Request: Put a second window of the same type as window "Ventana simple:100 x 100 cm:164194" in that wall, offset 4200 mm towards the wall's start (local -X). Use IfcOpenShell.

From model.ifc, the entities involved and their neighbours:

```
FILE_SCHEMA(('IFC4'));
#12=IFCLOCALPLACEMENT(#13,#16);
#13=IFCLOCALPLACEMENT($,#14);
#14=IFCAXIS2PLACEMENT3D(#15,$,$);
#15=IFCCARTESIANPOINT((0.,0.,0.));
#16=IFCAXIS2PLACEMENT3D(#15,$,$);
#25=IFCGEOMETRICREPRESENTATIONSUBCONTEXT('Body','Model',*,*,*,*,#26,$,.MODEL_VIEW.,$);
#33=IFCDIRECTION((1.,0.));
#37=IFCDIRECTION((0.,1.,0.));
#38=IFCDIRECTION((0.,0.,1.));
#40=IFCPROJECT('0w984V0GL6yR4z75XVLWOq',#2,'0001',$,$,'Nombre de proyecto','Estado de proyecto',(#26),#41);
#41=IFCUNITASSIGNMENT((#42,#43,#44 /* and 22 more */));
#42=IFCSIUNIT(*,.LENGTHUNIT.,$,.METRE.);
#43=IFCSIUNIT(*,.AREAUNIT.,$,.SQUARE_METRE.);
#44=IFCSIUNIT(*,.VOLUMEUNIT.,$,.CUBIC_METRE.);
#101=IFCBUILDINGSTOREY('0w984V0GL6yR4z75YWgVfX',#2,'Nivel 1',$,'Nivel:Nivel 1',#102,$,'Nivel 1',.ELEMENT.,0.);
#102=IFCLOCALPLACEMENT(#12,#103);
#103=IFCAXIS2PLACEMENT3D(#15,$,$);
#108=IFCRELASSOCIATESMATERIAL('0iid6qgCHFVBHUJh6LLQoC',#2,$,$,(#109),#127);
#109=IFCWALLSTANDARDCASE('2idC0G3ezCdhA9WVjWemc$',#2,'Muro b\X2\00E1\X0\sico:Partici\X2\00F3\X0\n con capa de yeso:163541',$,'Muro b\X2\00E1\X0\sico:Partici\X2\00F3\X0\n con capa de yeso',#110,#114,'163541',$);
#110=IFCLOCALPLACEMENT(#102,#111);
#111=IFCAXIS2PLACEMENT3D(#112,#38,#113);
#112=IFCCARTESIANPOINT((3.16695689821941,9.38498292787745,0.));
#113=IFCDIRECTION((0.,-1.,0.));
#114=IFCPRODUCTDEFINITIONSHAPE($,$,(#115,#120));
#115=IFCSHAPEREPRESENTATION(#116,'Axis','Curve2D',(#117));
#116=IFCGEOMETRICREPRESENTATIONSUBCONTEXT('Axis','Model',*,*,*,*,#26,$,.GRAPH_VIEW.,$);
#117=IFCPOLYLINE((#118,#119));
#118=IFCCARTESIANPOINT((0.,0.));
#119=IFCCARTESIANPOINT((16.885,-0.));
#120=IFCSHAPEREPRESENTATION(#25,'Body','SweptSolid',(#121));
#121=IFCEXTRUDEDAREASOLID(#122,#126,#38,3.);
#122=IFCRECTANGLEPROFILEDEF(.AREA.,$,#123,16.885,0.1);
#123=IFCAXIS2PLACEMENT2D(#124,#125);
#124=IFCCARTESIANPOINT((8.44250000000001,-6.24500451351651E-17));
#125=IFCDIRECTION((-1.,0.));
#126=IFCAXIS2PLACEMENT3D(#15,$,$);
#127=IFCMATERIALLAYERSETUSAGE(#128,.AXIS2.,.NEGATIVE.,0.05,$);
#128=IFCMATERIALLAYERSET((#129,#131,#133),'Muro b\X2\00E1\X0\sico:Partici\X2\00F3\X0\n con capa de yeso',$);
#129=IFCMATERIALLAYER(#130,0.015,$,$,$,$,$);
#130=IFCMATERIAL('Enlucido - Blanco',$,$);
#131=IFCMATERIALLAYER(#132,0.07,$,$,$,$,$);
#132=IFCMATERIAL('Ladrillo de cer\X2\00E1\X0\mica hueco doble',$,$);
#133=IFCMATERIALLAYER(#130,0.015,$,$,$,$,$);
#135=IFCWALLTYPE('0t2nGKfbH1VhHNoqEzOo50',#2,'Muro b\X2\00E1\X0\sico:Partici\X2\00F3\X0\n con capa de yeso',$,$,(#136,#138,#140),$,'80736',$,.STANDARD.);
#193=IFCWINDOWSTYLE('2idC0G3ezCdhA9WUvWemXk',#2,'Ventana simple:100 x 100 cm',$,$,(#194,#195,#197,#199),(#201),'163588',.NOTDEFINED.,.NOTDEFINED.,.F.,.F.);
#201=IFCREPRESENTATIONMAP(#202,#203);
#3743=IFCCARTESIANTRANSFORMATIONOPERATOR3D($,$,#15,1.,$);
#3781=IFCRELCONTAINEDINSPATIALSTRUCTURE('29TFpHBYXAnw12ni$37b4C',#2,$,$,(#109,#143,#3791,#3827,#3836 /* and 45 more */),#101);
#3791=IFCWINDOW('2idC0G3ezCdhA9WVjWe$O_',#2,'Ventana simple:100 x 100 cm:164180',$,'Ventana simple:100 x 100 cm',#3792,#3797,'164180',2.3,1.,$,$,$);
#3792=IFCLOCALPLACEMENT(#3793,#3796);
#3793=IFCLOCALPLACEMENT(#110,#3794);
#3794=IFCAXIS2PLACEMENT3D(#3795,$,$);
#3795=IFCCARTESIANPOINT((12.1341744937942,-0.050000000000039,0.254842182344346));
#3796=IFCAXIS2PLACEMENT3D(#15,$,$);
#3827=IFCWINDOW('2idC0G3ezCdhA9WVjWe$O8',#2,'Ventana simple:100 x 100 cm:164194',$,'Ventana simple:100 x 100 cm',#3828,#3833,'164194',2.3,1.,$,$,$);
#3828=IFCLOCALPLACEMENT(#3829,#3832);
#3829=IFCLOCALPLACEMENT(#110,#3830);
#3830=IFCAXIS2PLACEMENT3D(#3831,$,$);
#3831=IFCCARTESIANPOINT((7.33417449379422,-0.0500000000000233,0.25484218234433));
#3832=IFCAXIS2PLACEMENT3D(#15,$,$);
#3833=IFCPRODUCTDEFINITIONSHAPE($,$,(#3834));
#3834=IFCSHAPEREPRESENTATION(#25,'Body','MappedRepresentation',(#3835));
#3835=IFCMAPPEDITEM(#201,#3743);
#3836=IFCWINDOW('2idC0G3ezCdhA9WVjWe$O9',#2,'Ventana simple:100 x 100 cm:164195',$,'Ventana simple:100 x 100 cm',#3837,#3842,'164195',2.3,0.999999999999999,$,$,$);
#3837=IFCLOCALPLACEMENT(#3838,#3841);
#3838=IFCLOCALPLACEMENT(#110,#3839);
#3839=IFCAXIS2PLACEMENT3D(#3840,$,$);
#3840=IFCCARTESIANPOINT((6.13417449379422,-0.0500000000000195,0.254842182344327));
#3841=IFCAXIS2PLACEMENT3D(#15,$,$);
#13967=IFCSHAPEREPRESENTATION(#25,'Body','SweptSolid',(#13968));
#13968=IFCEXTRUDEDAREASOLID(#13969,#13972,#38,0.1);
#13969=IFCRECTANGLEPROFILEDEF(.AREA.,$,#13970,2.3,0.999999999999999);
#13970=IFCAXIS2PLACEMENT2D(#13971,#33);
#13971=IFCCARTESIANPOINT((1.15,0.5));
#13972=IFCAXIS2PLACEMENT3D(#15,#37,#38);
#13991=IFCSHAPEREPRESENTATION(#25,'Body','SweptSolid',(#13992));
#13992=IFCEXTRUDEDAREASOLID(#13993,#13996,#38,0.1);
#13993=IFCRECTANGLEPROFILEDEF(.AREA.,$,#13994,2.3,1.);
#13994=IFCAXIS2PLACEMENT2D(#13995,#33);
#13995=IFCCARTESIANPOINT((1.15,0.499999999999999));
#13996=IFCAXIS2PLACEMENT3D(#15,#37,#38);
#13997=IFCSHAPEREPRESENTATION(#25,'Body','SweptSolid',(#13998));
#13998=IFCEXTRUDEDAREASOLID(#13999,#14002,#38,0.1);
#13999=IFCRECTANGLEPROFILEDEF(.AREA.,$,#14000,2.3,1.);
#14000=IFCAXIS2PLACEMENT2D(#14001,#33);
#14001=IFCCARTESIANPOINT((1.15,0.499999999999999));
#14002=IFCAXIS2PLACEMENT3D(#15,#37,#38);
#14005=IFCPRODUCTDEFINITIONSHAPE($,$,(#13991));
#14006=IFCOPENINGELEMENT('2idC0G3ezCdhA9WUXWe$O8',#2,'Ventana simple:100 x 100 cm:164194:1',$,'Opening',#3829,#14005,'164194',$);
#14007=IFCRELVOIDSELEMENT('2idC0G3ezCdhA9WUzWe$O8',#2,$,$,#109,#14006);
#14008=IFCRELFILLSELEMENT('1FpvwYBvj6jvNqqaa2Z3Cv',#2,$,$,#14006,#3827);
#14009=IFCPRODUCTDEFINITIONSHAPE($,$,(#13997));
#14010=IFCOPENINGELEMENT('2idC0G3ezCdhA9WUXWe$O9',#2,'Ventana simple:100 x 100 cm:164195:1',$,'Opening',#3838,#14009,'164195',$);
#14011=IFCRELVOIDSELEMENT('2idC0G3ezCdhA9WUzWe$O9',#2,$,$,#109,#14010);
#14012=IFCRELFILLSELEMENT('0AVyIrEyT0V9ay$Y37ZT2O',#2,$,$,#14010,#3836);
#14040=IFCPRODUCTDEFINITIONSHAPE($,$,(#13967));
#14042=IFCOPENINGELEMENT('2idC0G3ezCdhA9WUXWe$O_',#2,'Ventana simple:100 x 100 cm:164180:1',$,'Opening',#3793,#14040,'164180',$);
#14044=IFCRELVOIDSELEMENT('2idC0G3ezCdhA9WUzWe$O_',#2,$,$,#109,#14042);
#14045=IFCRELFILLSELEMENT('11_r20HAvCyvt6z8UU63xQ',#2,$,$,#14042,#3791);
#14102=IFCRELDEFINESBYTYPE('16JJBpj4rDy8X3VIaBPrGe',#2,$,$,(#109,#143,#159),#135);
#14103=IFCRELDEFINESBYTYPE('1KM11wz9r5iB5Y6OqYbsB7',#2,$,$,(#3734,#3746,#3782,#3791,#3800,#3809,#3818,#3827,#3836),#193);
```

```python
import ifcopenshell
import ifcopenshell.api.feature
import ifcopenshell.api.geometry
import ifcopenshell.api.root
import ifcopenshell.geom
import ifcopenshell.util.element
import ifcopenshell.util.placement
import ifcopenshell.util.shape
import ifcopenshell.util.unit

model = ifcopenshell.open("model.ifc")
unit_scale = ifcopenshell.util.unit.calculate_unit_scale(model)
settings = ifcopenshell.geom.settings()


def volume(element):
    """Net volume in cubic metres, openings subtracted."""
    shape = ifcopenshell.geom.create_shape(settings, element)
    return ifcopenshell.util.shape.get_volume(shape.geometry)


def reuse_history(source, copy):
    """copy_class also copies each property set's owner history, people and application; keep the originals."""
    for rel in copy.IsDefinedBy:
        if rel.is_a("IfcRelDefinesByProperties") and (history := rel.RelatingPropertyDefinition.OwnerHistory):
            rel.RelatingPropertyDefinition.OwnerHistory = source.OwnerHistory
            ifcopenshell.util.element.remove_deep2(model, history)


window = model.by_guid("2idC0G3ezCdhA9WVjWe$O8")
opening = window.FillsVoids[0].RelatingOpeningElement
wall = opening.VoidsElements[0].RelatingBuildingElement
before = volume(wall)
shift = ifcopenshell.util.placement.get_local_placement(wall.ObjectPlacement)[:3, 0] * -4.2 / unit_scale

# copy_class copies the void relationship, type, container and properties, but no geometry.
new_opening = ifcopenshell.api.root.copy_class(model, product=opening)
new_opening.Representation = ifcopenshell.util.element.copy_deep(
    model, opening.Representation, exclude=["IfcGeometricRepresentationContext", "IfcRepresentationMap"]
)
new_opening.Name = "Ventana simple:100 x 100 cm"
new_opening.Tag = None
new_window = ifcopenshell.api.root.copy_class(model, product=window)
new_window.Representation = ifcopenshell.util.element.copy_deep(
    model, window.Representation, exclude=["IfcGeometricRepresentationContext", "IfcRepresentationMap"]
)
new_window.Name = "Ventana simple:100 x 100 cm"
new_window.Tag = None
reuse_history(window, new_window)
ifcopenshell.api.feature.add_filling(model, opening=new_opening, element=new_window)

for old, new in ((opening, new_opening), (window, new_window)):
    matrix = ifcopenshell.util.placement.get_local_placement(old.ObjectPlacement)
    matrix[:3, 3] += shift
    ifcopenshell.api.geometry.edit_object_placement(model, product=new, matrix=matrix, is_si=False)

after = volume(wall)

print(f"wall volume {before:.3f} -> {after:.3f} m3")

model.write("model_v2.ifc")
```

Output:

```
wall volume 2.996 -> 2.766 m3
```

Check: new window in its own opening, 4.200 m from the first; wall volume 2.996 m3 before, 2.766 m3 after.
